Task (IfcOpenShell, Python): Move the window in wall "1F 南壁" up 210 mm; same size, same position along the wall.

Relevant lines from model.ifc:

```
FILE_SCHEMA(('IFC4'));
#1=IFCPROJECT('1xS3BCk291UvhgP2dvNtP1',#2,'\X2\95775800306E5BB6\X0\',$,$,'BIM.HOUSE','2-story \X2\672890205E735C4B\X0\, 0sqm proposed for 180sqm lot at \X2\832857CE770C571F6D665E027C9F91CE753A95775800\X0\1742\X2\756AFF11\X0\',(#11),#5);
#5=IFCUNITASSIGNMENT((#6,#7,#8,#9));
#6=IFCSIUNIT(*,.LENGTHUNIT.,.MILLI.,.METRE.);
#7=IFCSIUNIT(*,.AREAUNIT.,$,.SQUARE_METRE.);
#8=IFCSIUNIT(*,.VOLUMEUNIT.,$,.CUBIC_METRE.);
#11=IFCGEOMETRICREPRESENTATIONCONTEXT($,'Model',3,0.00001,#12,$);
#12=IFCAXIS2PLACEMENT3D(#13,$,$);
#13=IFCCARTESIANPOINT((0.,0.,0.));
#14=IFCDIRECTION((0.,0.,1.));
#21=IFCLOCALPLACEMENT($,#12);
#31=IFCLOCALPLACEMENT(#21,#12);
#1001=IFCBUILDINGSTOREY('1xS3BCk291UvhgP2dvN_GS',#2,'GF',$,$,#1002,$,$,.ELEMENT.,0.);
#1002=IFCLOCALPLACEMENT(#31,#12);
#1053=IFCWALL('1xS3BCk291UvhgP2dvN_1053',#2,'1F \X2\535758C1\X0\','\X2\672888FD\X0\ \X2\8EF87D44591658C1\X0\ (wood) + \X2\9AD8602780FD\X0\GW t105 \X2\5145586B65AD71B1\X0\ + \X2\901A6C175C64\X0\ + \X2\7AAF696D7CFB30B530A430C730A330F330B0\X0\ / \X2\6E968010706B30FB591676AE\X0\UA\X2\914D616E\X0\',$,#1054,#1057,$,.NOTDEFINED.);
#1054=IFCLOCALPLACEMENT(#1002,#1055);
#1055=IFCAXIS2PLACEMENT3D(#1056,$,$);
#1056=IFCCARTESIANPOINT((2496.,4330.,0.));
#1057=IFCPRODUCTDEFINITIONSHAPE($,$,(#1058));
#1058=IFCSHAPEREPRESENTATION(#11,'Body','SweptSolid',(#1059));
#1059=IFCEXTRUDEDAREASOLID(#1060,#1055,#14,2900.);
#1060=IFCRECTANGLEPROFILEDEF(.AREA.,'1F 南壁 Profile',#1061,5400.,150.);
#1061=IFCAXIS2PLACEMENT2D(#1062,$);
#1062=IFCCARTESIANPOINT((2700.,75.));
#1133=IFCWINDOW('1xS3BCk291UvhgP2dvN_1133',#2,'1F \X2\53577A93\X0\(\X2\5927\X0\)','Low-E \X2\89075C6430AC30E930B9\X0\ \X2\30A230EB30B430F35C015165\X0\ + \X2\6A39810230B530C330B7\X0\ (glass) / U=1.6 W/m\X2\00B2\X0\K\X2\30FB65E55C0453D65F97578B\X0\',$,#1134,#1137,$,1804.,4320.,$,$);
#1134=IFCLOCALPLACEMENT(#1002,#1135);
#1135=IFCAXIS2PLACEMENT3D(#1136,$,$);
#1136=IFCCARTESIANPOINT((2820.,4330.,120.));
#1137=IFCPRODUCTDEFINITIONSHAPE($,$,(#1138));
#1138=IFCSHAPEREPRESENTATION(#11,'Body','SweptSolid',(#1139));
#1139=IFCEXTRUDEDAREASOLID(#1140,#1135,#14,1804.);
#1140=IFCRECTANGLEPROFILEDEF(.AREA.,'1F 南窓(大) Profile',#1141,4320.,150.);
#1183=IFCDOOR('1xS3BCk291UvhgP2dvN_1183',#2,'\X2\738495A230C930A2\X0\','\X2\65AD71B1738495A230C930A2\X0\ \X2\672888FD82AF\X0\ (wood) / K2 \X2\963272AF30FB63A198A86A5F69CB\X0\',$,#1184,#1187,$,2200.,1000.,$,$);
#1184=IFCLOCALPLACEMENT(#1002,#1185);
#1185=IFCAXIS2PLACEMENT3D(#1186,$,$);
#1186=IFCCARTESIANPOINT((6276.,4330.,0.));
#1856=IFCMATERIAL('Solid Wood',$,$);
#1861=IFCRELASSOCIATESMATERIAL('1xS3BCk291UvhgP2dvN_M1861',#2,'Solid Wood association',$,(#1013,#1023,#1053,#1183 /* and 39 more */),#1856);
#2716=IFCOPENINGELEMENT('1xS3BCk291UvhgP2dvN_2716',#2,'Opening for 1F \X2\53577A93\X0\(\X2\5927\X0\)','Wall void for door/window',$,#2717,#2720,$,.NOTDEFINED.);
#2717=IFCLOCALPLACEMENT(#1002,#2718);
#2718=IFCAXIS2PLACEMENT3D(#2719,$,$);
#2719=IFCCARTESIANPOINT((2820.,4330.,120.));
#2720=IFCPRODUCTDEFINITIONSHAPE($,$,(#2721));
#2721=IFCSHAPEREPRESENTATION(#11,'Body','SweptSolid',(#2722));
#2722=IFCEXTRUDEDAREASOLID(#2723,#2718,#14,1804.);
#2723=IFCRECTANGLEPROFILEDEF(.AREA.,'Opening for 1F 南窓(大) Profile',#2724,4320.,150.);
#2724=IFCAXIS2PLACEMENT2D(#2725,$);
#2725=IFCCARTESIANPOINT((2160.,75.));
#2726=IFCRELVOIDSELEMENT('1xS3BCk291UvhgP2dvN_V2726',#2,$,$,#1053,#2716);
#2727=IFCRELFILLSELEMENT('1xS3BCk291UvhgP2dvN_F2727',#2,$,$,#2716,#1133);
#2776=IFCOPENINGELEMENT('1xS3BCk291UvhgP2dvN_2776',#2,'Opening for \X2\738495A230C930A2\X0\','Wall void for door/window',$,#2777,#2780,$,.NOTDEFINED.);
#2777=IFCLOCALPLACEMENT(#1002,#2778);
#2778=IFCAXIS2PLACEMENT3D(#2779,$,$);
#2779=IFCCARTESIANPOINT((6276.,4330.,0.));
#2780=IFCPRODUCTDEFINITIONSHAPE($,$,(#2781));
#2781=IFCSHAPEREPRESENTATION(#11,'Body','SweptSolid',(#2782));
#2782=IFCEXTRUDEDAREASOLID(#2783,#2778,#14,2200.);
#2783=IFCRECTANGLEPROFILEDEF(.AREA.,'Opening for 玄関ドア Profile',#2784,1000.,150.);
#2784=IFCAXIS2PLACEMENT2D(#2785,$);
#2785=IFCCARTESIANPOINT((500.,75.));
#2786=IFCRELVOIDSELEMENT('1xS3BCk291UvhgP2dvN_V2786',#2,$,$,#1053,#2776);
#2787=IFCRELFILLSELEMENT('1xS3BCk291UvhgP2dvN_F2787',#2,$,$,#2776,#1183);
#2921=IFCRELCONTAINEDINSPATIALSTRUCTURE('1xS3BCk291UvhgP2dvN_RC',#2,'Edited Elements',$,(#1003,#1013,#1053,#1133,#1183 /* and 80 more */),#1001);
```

```python
import numpy as np
import ifcopenshell
import ifcopenshell.api.geometry
import ifcopenshell.util.placement
import ifcopenshell.util.unit

model = ifcopenshell.open("model.ifc")
unit_scale = ifcopenshell.util.unit.calculate_unit_scale(model)

window = model.by_guid("1xS3BCk291UvhgP2dvN_1133")
opening = window.FillsVoids[0].RelatingOpeningElement
dz = 0.21 / unit_scale

shift = np.array([0.0, 0.0, dz])
# The window is not placed relative to its opening, so move both.
for product in (opening, window):
    matrix = ifcopenshell.util.placement.get_local_placement(product.ObjectPlacement)
    matrix[:3, 3] += shift
    ifcopenshell.api.geometry.edit_object_placement(model, product=product, matrix=matrix, is_si=False)

print(f"moved by {dz * unit_scale:+.3f} m")

model.write("model_updated.ifc")
```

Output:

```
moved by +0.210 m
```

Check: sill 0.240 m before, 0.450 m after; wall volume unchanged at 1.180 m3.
